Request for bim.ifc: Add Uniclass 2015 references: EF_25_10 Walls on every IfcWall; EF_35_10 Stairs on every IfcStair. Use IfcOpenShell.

First a look at what the model holds.

```python
import ifcopenshell

model = ifcopenshell.open("bim.ifc")
print(model.schema)
print("classifications:", [c.Name for c in model.by_type("IfcClassification")])
for ifc_class in ("IfcDoor", "IfcRoof", "IfcStair", "IfcWall", "IfcWindow"):
    print(ifc_class, len(model.by_type(ifc_class)))
```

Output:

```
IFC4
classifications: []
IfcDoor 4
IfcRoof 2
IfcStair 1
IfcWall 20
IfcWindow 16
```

```python
import ifcopenshell
import ifcopenshell.api.classification

model = ifcopenshell.open("bim.ifc")

system = ifcopenshell.api.classification.add_classification(model, classification="Uniclass 2015")

codes = {
    "IfcWall": ("EF_25_10", "Walls"),
    "IfcStair": ("EF_35_10", "Stairs"),
}
for ifc_class, (code, name) in codes.items():
    products = model.by_type(ifc_class)
    ifcopenshell.api.classification.add_reference(
        model, products=products, classification=system, identification=code, name=name
    )
    print(code, len(products))

model.write("bim_rev.ifc")
```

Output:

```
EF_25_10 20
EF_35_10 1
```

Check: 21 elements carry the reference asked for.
